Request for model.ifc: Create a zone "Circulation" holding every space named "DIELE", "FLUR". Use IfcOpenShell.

First a look at what the model holds.

```python
import ifcopenshell

model = ifcopenshell.open("model.ifc")
print(model.schema)
seen = {}
for space in model.by_type("IfcSpace"):
    seen[space.LongName] = seen.get(space.LongName, 0) + 1
for name, count in sorted(seen.items(), key=str):
    print(count, "x", name)
print("zones:", [z.Name for z in model.by_type("IfcZone")][:20])
```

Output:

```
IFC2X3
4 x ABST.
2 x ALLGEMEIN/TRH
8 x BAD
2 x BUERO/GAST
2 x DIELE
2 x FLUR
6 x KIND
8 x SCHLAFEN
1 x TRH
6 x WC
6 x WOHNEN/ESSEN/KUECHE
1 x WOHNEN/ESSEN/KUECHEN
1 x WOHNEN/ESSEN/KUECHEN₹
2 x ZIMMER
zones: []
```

```python
import ifcopenshell
import ifcopenshell.api.group
import ifcopenshell.api.root

model = ifcopenshell.open("model.ifc")

names = {"DIELE", "FLUR"}
spaces = [s for s in model.by_type("IfcSpace") if s.LongName in names]

zone = ifcopenshell.api.root.create_entity(model, ifc_class="IfcZone", name="Circulation")
ifcopenshell.api.group.assign_group(model, products=spaces, group=zone)
print(len(spaces), "spaces in", zone.Name)

model.write("model-out.ifc")
```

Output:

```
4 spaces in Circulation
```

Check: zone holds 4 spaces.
